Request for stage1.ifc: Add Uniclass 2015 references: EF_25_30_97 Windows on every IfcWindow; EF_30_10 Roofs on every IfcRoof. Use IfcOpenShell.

First a look at what the model holds.

```python
import ifcopenshell

model = ifcopenshell.open("stage1.ifc")
print(model.schema)
print("classifications:", [c.Name for c in model.by_type("IfcClassification")])
for ifc_class in ("IfcDoor", "IfcRoof", "IfcStair", "IfcWall", "IfcWindow"):
    print(ifc_class, len(model.by_type(ifc_class)))
```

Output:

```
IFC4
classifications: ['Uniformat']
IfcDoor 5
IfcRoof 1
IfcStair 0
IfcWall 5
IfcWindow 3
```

```python
import ifcopenshell
import ifcopenshell.api.classification

model = ifcopenshell.open("stage1.ifc")

system = ifcopenshell.api.classification.add_classification(model, classification="Uniclass 2015")

codes = {
    "IfcWindow": ("EF_25_30_97", "Windows"),
    "IfcRoof": ("EF_30_10", "Roofs"),
}
for ifc_class, (code, name) in codes.items():
    products = model.by_type(ifc_class)
    ifcopenshell.api.classification.add_reference(
        model, products=products, classification=system, identification=code, name=name
    )
    print(code, len(products))

model.write("stage1-out.ifc")
```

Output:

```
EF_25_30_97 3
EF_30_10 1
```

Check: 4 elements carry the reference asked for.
